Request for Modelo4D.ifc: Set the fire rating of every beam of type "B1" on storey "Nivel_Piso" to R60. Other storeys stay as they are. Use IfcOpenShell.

First a look at what the model holds.

```python
import ifcopenshell
import ifcopenshell.util.element

model = ifcopenshell.open("Modelo4D.ifc")
print(model.schema)
storey = next(s for s in model.by_type("IfcBuildingStorey") if s.Name == "Nivel_Piso")
beams = [e for e in ifcopenshell.util.element.get_decomposition(storey) if e.is_a("IfcBeam")]
seen = {}
for e in beams:
    element_type = ifcopenshell.util.element.get_type(e)
    key = (element_type.Name if element_type != e and element_type else None, ifcopenshell.util.element.get_pset(e, "Pset_BeamCommon", "FireRating"))
    seen[key] = seen.get(key, 0) + 1
for (name, value), count in sorted(seen.items(), key=str):
    print(count, "x", name, "|", value)
```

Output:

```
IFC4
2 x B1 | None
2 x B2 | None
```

```python
import ifcopenshell
import ifcopenshell.api.pset
import ifcopenshell.util.element

model = ifcopenshell.open("Modelo4D.ifc")

storey = next(s for s in model.by_type("IfcBuildingStorey") if s.Name == "Nivel_Piso")
beams = [e for e in ifcopenshell.util.element.get_decomposition(storey) if e.is_a("IfcBeam")]

count = 0
for e in beams:
    element_type = ifcopenshell.util.element.get_type(e)
    if element_type in (None, e) or element_type.Name != "B1":
        continue
    # add_pset returns the element's existing set when there is one.
    pset = ifcopenshell.api.pset.add_pset(model, product=e, name="Pset_BeamCommon")
    ifcopenshell.api.pset.edit_pset(model, pset=pset, properties={"FireRating": "R60"})
    count += 1

print(count, "beams updated")

model.write("Modelo4D_edited.ifc")
```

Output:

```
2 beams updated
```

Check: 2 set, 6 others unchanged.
